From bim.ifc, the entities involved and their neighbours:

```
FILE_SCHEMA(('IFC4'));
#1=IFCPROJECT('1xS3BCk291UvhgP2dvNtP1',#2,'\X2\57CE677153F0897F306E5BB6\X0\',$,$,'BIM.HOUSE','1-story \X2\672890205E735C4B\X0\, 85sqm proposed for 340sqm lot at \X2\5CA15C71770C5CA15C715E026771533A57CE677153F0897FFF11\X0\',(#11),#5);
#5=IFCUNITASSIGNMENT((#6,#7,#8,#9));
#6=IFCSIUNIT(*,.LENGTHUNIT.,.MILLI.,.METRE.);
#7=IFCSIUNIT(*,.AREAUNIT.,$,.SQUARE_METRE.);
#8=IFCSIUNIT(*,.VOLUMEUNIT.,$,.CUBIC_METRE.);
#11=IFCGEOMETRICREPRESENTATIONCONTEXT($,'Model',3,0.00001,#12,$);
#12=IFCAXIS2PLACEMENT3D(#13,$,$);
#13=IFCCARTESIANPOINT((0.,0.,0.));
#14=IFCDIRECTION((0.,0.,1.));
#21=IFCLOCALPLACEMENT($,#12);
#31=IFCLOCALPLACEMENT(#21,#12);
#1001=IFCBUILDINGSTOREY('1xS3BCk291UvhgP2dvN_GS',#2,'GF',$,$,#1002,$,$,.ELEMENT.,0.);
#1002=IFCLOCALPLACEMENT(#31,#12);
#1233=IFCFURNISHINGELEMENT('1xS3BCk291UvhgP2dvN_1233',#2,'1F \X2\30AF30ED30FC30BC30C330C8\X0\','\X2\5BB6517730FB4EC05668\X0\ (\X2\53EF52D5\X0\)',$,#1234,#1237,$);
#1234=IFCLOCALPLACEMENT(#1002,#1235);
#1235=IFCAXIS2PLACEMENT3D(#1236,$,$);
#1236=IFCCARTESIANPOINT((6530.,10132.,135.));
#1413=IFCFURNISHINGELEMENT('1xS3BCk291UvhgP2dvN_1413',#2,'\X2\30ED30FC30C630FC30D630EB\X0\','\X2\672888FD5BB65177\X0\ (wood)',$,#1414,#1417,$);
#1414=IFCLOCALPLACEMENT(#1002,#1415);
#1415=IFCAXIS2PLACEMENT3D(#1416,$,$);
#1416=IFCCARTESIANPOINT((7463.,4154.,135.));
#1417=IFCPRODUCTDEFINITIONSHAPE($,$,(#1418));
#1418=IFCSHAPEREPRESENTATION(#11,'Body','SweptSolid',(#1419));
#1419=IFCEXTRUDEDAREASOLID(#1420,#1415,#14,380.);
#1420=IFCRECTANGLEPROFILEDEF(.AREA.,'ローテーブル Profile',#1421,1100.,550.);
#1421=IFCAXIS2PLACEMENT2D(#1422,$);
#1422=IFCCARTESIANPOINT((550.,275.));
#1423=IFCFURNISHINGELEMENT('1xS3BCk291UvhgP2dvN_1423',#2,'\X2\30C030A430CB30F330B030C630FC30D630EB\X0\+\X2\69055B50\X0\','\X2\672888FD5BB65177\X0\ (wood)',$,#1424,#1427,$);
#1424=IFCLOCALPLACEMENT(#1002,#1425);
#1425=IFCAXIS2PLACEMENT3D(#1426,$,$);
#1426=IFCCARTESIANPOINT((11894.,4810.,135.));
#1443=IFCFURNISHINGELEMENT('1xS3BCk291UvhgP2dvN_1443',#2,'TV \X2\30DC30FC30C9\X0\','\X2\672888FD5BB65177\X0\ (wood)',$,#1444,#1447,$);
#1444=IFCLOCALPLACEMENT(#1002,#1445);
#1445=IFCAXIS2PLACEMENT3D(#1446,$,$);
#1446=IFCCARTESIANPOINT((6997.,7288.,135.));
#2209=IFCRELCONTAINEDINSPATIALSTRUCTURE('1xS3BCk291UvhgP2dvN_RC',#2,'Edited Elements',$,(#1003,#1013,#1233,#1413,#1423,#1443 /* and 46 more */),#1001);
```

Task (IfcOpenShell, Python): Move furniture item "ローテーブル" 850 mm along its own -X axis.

```python
import ifcopenshell
import ifcopenshell.api.geometry
import ifcopenshell.util.placement

model = ifcopenshell.open("bim.ifc")

item = model.by_id(1413)
matrix = ifcopenshell.util.placement.get_local_placement(item.ObjectPlacement)
matrix[:3, 3] -= matrix[:3, 0] * 850.0
ifcopenshell.api.geometry.edit_object_placement(model, product=item, matrix=matrix, is_si=False)

print(ifcopenshell.util.placement.get_local_placement(item.ObjectPlacement).round(3) + 0.0)

model.write("bim_updated.ifc")
```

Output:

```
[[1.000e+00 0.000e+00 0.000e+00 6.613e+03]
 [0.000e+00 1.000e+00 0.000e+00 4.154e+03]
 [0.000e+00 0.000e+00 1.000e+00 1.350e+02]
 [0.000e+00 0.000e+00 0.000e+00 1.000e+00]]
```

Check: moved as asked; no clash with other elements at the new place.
